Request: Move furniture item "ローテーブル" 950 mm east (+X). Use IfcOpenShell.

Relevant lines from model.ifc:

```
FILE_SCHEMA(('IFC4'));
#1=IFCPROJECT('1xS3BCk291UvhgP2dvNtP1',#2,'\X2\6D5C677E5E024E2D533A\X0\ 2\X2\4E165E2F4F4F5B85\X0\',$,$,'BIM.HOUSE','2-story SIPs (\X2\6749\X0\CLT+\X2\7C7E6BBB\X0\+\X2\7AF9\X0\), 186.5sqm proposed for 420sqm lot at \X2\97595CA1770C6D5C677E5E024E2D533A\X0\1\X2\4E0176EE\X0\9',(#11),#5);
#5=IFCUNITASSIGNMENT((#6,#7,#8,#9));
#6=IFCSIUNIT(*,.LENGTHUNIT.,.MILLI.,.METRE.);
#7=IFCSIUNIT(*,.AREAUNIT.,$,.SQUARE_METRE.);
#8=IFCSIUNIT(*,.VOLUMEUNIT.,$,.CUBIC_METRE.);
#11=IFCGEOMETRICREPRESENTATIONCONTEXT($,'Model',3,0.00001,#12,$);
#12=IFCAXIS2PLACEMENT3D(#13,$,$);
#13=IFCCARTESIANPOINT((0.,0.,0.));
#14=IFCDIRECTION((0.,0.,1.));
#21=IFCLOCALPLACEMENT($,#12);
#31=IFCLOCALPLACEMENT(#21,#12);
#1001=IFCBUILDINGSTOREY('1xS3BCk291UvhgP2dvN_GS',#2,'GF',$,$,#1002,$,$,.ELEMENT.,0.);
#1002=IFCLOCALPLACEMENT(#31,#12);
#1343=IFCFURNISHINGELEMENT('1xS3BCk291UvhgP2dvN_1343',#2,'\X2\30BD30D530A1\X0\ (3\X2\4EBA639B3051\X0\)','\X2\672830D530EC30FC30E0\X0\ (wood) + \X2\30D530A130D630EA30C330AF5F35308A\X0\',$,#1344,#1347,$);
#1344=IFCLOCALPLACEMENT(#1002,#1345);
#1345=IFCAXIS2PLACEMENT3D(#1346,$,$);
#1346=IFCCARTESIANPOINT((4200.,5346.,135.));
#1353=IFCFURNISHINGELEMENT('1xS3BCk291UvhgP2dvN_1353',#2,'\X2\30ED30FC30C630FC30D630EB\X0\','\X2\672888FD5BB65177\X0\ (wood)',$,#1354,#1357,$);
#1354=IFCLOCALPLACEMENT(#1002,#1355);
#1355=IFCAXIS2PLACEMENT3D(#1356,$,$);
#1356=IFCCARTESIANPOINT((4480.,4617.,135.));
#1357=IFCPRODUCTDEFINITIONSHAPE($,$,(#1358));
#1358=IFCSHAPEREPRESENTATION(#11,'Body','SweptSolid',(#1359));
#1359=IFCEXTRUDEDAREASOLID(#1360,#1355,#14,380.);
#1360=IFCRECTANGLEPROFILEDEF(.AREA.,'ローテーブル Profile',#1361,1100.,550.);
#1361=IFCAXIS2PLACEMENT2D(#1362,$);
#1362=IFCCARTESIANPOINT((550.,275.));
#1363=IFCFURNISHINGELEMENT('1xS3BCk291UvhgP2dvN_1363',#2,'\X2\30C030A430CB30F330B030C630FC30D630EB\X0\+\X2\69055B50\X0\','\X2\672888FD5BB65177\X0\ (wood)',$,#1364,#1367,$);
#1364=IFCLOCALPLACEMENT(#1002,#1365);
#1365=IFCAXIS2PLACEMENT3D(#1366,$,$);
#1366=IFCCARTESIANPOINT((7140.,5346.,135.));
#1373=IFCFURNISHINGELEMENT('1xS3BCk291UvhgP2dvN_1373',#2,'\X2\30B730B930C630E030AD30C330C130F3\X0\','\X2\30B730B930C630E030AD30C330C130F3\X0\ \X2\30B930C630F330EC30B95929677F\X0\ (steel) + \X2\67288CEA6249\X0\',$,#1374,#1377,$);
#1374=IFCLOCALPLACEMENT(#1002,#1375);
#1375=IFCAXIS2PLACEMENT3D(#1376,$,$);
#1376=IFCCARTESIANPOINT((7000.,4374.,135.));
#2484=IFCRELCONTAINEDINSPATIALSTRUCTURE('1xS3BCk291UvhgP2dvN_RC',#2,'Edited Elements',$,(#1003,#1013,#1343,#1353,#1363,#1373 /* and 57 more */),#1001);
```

```python
import ifcopenshell
import ifcopenshell.api.geometry
import ifcopenshell.util.placement
import ifcopenshell.util.unit

model = ifcopenshell.open("model.ifc")
unit_scale = ifcopenshell.util.unit.calculate_unit_scale(model)

item = model.by_guid("1xS3BCk291UvhgP2dvN_1353")
matrix = ifcopenshell.util.placement.get_local_placement(item.ObjectPlacement)
matrix[0, 3] += 0.95 / unit_scale
ifcopenshell.api.geometry.edit_object_placement(model, product=item, matrix=matrix, is_si=False)

print(ifcopenshell.util.placement.get_local_placement(item.ObjectPlacement).round(3) + 0.0)

model.write("model_v2.ifc")
```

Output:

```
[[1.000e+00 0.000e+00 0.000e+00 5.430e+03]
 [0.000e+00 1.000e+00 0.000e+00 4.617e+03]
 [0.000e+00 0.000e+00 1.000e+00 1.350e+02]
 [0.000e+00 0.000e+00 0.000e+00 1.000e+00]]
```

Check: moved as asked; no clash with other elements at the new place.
